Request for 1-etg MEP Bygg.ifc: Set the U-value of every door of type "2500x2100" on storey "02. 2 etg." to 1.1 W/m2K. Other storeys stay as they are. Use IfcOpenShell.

First a look at what the model holds.

```python
import ifcopenshell
import ifcopenshell.util.element

model = ifcopenshell.open("1-etg MEP Bygg.ifc")
print(model.schema)
storey = next(s for s in model.by_type("IfcBuildingStorey") if s.Name == "02. 2 etg.")
doors = [e for e in ifcopenshell.util.element.get_decomposition(storey) if e.is_a("IfcDoor")]
seen = {}
for e in doors:
    element_type = ifcopenshell.util.element.get_type(e)
    key = (element_type.Name if element_type != e and element_type else None, ifcopenshell.util.element.get_pset(e, "Pset_DoorCommon", "ThermalTransmittance"))
    seen[key] = seen.get(key, 0) + 1
for (name, value), count in sorted(seen.items(), key=str):
    print(count, "x", name, "|", value)
```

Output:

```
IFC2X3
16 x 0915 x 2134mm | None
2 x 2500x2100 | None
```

```python
import ifcopenshell
import ifcopenshell.api.pset
import ifcopenshell.util.element

model = ifcopenshell.open("1-etg MEP Bygg.ifc")

storey = next(s for s in model.by_type("IfcBuildingStorey") if s.Name == "02. 2 etg.")
doors = [e for e in ifcopenshell.util.element.get_decomposition(storey) if e.is_a("IfcDoor")]

count = 0
for e in doors:
    element_type = ifcopenshell.util.element.get_type(e)
    if element_type in (None, e) or element_type.Name != "2500x2100":
        continue
    # add_pset returns the element's existing set when there is one.
    pset = ifcopenshell.api.pset.add_pset(model, product=e, name="Pset_DoorCommon")
    ifcopenshell.api.pset.edit_pset(model, pset=pset, properties={"ThermalTransmittance": 1.1})
    count += 1

print(count, "doors updated")

model.write("1-etg MEP Bygg_v2.ifc")
```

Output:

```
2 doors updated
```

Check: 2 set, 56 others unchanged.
